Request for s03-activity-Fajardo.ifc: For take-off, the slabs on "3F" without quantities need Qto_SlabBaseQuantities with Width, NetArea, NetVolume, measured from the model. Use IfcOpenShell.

First a look at what the model holds.

```python
import ifcopenshell
import ifcopenshell.util.element
import ifcopenshell.util.unit

model = ifcopenshell.open("s03-activity-Fajardo.ifc")
print(model.schema)
for unit_type in ("LENGTHUNIT", "AREAUNIT", "VOLUMEUNIT"):
    print(unit_type, ifcopenshell.util.unit.calculate_unit_scale(model, unit_type))
storey = next(s for s in model.by_type("IfcBuildingStorey") if s.Name == "3F")
slabs = [e for e in ifcopenshell.util.element.get_decomposition(storey) if e.is_a("IfcSlab")]
for e in sorted(slabs, key=lambda e: e.id()):
    print(e.id(), e.is_a(), e.Name, list(ifcopenshell.util.element.get_psets(e, qtos_only=True)), sep=" | ")
```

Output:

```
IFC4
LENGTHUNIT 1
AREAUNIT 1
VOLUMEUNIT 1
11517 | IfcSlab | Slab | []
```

```python
import ifcopenshell
import ifcopenshell.api.pset
import ifcopenshell.geom
import ifcopenshell.util.element
import ifcopenshell.util.shape
import ifcopenshell.util.unit

model = ifcopenshell.open("s03-activity-Fajardo.ifc")
unit_scale = ifcopenshell.util.unit.calculate_unit_scale(model)
area_scale = ifcopenshell.util.unit.calculate_unit_scale(model, "AREAUNIT")
volume_scale = ifcopenshell.util.unit.calculate_unit_scale(model, "VOLUMEUNIT")
settings = ifcopenshell.geom.settings()

storey = next(s for s in model.by_type("IfcBuildingStorey") if s.Name == "3F")
slabs = [e for e in ifcopenshell.util.element.get_decomposition(storey) if e.is_a("IfcSlab")]

for e in sorted(slabs, key=lambda e: e.id()):
    if ifcopenshell.util.element.get_psets(e, qtos_only=True, should_inherit=False):
        continue
    # Geometry comes back in metres, in the element's own axes.
    shape = ifcopenshell.geom.create_shape(settings, e)
    values = {
        "Width": ifcopenshell.util.shape.get_z(shape.geometry) / unit_scale,
        "NetArea": ifcopenshell.util.shape.get_footprint_area(shape.geometry) / area_scale,
        "NetVolume": ifcopenshell.util.shape.get_volume(shape.geometry) / volume_scale,
    }
    qto = ifcopenshell.api.pset.add_qto(model, product=e, name="Qto_SlabBaseQuantities")
    ifcopenshell.api.pset.edit_qto(model, qto=qto, properties=values)
    print(e.id(), {k: round(v, 3) for k, v in values.items()})

model.write("s03-activity-Fajardo_updated.ifc")
```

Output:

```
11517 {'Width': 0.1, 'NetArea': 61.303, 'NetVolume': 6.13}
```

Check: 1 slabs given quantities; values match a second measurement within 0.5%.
